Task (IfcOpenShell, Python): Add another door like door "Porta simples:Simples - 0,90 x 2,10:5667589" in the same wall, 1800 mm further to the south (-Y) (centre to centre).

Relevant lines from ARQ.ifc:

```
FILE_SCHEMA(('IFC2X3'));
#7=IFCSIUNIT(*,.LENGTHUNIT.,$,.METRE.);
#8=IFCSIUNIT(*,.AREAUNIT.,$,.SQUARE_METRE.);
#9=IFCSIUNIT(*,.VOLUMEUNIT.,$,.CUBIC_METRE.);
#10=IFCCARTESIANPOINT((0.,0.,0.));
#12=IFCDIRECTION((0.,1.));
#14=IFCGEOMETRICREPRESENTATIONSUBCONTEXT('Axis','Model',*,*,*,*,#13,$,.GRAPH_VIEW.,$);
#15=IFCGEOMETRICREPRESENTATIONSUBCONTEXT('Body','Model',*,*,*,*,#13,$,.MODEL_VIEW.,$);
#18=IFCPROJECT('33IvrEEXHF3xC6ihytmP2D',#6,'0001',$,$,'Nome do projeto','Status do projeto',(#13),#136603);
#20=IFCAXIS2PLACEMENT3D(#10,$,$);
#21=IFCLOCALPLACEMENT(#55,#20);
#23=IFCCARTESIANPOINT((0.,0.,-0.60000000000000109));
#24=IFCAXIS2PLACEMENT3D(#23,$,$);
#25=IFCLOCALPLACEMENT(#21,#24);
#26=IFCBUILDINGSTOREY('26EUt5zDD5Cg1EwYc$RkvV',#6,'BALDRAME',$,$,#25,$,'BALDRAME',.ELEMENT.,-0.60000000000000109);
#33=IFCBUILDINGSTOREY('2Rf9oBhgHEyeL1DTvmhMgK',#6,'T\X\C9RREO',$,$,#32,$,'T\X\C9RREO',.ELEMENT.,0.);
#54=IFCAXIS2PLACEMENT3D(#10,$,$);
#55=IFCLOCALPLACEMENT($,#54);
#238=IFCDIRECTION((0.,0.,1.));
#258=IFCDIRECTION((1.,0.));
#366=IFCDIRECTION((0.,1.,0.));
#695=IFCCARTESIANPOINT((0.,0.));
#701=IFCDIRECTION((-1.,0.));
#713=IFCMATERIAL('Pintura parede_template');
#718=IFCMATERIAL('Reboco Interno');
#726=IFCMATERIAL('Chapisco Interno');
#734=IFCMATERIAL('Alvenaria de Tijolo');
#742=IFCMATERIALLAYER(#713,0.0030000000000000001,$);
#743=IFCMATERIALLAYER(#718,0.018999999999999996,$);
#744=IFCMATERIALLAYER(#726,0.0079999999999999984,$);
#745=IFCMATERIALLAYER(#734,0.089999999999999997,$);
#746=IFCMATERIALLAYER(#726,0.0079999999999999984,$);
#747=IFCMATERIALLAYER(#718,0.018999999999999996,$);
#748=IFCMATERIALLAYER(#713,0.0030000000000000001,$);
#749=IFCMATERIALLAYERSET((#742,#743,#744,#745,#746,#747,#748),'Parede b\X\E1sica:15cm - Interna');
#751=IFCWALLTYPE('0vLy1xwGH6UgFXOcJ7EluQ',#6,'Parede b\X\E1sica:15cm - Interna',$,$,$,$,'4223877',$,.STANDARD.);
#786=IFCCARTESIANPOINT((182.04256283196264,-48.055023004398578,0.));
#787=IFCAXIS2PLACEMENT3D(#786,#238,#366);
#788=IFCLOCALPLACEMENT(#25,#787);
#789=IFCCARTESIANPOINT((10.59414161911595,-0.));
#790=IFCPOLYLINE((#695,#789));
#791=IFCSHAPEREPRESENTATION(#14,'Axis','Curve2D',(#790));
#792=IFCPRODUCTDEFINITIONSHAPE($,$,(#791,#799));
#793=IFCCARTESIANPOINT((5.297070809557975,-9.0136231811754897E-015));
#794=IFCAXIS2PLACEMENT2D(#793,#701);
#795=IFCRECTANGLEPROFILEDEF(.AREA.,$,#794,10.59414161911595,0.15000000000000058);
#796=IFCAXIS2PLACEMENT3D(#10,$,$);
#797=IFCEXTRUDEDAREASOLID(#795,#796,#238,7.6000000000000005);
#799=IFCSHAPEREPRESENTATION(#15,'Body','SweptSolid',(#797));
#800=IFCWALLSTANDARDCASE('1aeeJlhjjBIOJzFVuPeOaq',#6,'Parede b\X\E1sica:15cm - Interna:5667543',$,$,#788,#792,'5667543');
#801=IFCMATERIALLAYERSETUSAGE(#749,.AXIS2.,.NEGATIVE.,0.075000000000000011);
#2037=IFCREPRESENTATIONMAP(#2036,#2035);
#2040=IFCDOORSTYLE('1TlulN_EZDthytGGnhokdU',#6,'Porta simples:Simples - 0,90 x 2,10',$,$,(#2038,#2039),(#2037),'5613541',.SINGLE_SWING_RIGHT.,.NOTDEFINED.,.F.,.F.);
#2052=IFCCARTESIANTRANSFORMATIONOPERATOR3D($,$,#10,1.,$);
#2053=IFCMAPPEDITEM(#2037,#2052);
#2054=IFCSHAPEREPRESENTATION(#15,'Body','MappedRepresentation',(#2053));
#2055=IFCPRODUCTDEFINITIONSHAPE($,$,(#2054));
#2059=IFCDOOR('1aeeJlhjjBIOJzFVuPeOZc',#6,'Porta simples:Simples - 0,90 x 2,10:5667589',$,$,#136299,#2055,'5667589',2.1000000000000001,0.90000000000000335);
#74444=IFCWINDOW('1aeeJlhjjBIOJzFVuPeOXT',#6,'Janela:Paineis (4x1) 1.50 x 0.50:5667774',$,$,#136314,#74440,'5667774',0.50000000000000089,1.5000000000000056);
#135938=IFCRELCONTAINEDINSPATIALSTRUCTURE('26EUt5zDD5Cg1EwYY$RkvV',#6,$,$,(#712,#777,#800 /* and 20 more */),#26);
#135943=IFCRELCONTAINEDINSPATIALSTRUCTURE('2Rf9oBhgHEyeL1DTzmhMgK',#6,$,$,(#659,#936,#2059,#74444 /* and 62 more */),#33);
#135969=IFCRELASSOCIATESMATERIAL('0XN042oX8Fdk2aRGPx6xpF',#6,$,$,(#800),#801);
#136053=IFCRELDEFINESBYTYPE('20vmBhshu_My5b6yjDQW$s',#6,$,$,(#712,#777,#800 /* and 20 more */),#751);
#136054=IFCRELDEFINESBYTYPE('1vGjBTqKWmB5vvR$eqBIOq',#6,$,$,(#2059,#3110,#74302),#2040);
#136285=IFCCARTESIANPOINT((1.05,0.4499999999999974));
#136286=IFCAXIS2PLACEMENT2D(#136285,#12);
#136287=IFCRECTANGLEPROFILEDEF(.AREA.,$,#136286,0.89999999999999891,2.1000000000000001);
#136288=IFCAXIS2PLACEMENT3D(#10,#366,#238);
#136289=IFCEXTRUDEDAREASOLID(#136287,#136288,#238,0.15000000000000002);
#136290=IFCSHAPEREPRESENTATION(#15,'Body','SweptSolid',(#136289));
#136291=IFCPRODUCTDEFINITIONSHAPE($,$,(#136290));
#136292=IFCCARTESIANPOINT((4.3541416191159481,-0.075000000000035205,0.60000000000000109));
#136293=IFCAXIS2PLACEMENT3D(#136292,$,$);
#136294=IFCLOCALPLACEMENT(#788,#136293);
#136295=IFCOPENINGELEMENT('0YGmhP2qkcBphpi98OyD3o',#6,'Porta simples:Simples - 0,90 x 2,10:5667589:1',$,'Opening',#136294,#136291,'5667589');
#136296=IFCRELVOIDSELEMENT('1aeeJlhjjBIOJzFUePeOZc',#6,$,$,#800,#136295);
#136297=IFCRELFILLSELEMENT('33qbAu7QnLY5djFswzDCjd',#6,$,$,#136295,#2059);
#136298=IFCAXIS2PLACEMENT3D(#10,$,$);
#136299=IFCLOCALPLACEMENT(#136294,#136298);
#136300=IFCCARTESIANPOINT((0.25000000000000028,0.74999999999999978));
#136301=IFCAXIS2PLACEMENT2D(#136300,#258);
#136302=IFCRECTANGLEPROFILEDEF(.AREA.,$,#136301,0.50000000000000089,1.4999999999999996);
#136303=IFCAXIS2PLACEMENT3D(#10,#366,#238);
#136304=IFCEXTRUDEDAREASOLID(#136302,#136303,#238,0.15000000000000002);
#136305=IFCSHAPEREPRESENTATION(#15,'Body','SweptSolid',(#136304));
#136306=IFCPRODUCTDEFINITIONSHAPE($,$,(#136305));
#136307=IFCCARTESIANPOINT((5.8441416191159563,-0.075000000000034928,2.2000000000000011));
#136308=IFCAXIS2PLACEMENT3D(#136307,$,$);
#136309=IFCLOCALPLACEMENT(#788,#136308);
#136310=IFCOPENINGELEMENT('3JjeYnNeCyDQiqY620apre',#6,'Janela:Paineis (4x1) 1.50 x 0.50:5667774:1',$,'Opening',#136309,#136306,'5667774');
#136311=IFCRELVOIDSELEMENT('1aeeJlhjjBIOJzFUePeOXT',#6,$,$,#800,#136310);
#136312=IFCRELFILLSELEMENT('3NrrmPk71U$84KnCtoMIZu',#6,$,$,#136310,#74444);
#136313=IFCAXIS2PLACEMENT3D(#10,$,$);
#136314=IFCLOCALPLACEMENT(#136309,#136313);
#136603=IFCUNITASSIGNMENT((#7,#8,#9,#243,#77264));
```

```python
import ifcopenshell
import ifcopenshell.api.feature
import ifcopenshell.api.geometry
import ifcopenshell.api.root
import ifcopenshell.geom
import ifcopenshell.util.element
import ifcopenshell.util.placement
import ifcopenshell.util.shape
import ifcopenshell.util.unit

model = ifcopenshell.open("ARQ.ifc")
unit_scale = ifcopenshell.util.unit.calculate_unit_scale(model)
settings = ifcopenshell.geom.settings()


def volume(element):
    """Net volume in cubic metres, openings subtracted."""
    shape = ifcopenshell.geom.create_shape(settings, element)
    return ifcopenshell.util.shape.get_volume(shape.geometry)


def reuse_history(source, copy):
    """copy_class also copies each property set's owner history, people and application; keep the originals."""
    for rel in copy.IsDefinedBy:
        if rel.is_a("IfcRelDefinesByProperties") and (history := rel.RelatingPropertyDefinition.OwnerHistory):
            rel.RelatingPropertyDefinition.OwnerHistory = source.OwnerHistory
            ifcopenshell.util.element.remove_deep2(model, history)


door = model.by_id(2059)
opening = door.FillsVoids[0].RelatingOpeningElement
wall = opening.VoidsElements[0].RelatingBuildingElement
before = volume(wall)
shift = ifcopenshell.util.placement.get_local_placement(wall.ObjectPlacement)[:3, 0] * -1.8 / unit_scale

# copy_class copies the void relationship, type, container and properties, but no geometry.
new_opening = ifcopenshell.api.root.copy_class(model, product=opening)
new_opening.Representation = ifcopenshell.util.element.copy_deep(
    model, opening.Representation, exclude=["IfcGeometricRepresentationContext", "IfcRepresentationMap"]
)
new_opening.Name = "Porta simples:Simples - 0,90 x 2,10"
new_opening.Tag = None
new_door = ifcopenshell.api.root.copy_class(model, product=door)
new_door.Representation = ifcopenshell.util.element.copy_deep(
    model, door.Representation, exclude=["IfcGeometricRepresentationContext", "IfcRepresentationMap"]
)
new_door.Name = "Porta simples:Simples - 0,90 x 2,10"
new_door.Tag = None
reuse_history(door, new_door)
fills = ifcopenshell.api.feature.add_filling(model, opening=new_opening, element=new_door)
fills.OwnerHistory = new_door.OwnerHistory  # required in IFC2X3

for old, new in ((opening, new_opening), (door, new_door)):
    matrix = ifcopenshell.util.placement.get_local_placement(old.ObjectPlacement)
    matrix[:3, 3] += shift
    ifcopenshell.api.geometry.edit_object_placement(model, product=new, matrix=matrix, is_si=False)

after = volume(wall)

print(f"wall volume {before:.3f} -> {after:.3f} m3")

model.write("ARQ_edited.ifc")
```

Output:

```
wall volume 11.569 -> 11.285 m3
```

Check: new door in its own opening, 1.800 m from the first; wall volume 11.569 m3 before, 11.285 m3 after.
